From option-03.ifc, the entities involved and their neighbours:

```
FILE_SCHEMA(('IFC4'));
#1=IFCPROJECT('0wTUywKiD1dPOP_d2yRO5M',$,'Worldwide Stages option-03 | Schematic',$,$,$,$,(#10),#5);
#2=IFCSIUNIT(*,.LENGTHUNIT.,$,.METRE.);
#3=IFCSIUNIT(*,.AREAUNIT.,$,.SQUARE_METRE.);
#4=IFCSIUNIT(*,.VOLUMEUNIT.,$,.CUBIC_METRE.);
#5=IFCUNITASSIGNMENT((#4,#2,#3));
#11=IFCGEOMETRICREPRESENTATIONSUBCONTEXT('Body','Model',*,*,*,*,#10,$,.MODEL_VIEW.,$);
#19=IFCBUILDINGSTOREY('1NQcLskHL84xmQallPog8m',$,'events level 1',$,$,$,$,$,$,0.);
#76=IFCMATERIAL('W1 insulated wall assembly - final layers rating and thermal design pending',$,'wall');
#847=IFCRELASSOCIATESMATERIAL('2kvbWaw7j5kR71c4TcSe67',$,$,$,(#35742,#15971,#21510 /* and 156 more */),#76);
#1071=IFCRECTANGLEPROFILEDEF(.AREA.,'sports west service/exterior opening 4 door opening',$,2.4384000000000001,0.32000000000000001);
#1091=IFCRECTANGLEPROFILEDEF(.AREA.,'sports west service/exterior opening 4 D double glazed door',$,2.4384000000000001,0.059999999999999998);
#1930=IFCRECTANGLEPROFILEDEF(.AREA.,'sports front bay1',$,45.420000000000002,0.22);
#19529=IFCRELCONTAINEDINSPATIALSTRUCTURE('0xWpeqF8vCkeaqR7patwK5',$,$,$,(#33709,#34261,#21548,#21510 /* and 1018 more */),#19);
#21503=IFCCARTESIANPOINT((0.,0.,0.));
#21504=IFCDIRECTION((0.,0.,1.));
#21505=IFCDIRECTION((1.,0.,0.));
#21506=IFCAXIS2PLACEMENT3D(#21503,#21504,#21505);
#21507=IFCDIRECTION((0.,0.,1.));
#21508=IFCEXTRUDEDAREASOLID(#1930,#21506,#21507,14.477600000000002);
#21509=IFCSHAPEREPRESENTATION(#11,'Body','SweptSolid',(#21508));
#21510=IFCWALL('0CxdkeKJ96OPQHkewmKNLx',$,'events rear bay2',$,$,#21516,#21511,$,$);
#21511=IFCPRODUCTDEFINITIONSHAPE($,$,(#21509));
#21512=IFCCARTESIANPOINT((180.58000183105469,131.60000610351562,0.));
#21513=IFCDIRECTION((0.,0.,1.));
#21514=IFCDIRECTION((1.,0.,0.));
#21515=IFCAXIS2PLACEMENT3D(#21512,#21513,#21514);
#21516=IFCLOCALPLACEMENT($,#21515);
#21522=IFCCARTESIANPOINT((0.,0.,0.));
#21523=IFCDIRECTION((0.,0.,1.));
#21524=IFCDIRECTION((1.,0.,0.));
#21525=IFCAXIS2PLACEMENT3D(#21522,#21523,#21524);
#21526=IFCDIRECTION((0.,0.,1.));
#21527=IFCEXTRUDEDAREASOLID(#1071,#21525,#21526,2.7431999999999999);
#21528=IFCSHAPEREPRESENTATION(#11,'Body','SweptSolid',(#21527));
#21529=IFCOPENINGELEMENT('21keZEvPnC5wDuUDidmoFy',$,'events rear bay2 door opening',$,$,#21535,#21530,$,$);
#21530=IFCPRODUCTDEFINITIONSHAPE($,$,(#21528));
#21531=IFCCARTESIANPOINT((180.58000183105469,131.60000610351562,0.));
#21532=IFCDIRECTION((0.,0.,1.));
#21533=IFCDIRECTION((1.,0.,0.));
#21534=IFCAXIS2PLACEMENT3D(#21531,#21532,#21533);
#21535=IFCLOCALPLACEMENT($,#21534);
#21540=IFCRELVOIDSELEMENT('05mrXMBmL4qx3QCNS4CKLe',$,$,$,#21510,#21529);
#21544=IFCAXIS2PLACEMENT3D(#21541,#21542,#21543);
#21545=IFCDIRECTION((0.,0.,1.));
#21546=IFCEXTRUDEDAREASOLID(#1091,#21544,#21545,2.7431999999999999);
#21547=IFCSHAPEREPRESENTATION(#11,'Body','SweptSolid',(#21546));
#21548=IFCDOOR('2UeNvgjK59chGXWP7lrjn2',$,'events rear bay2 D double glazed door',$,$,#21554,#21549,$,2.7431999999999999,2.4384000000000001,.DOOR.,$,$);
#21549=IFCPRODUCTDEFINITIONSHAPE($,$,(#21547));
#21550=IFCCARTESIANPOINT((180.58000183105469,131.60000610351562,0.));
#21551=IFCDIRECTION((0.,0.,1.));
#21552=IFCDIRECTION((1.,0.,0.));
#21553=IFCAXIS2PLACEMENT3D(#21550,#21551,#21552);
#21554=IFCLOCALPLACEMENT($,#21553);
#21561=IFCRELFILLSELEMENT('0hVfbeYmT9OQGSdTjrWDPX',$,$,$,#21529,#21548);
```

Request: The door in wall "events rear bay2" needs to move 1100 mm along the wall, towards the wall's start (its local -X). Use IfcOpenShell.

```python
import ifcopenshell
import ifcopenshell.api.geometry
import ifcopenshell.util.placement
import ifcopenshell.util.unit

model = ifcopenshell.open("option-03.ifc")
unit_scale = ifcopenshell.util.unit.calculate_unit_scale(model)

door = model.by_guid("2UeNvgjK59chGXWP7lrjn2")
opening = door.FillsVoids[0].RelatingOpeningElement
wall = opening.VoidsElements[0].RelatingBuildingElement

wall_matrix = ifcopenshell.util.placement.get_local_placement(wall.ObjectPlacement)
shift = wall_matrix[:3, 0] * -1.1 / unit_scale
before = ifcopenshell.util.placement.get_local_placement(door.ObjectPlacement)[:3, 3].copy()

# The door is not placed relative to its opening, so move both.
for product in (opening, door):
    matrix = ifcopenshell.util.placement.get_local_placement(product.ObjectPlacement)
    matrix[:3, 3] += shift
    ifcopenshell.api.geometry.edit_object_placement(model, product=product, matrix=matrix, is_si=False)

after = ifcopenshell.util.placement.get_local_placement(door.ObjectPlacement)[:3, 3]
print("door moved by", (after - before).round(3) + 0.0)

model.write("option-03_v2.ifc")
```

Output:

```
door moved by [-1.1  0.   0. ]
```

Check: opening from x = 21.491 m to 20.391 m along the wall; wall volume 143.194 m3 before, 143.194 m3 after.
